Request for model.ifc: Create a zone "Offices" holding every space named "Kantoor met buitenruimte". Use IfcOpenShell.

First a look at what the model holds.

```python
import ifcopenshell

model = ifcopenshell.open("model.ifc")
print(model.schema)
seen = {}
for space in model.by_type("IfcSpace"):
    seen[space.LongName] = seen.get(space.LongName, 0) + 1
for name, count in sorted(seen.items(), key=str):
    print(count, "x", name)
print("zones:", [z.Name for z in model.by_type("IfcZone")][:20])
```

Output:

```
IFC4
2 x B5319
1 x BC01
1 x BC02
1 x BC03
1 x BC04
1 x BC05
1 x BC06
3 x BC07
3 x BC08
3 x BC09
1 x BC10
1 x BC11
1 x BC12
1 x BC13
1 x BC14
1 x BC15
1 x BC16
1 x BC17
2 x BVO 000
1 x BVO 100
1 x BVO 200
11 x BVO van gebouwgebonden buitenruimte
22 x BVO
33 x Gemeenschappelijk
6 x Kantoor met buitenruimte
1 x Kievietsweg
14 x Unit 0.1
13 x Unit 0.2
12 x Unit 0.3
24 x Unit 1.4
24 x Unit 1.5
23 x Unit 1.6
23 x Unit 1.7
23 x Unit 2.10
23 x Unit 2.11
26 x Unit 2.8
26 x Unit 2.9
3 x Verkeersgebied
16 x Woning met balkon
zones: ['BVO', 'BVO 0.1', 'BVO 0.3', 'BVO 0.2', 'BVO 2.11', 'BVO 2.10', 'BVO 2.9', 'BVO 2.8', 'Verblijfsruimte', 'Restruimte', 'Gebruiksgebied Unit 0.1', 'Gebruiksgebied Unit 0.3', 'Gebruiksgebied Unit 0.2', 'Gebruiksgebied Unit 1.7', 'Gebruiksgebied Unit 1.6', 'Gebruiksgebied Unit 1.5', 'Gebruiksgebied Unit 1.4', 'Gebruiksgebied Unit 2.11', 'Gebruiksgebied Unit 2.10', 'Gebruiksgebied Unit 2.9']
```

```python
import ifcopenshell
import ifcopenshell.api.group
import ifcopenshell.api.root

model = ifcopenshell.open("model.ifc")

names = {"Kantoor met buitenruimte"}
spaces = [s for s in model.by_type("IfcSpace") if s.LongName in names]

zone = ifcopenshell.api.root.create_entity(model, ifc_class="IfcZone", name="Offices")
ifcopenshell.api.group.assign_group(model, products=spaces, group=zone)
print(len(spaces), "spaces in", zone.Name)

model.write("model_updated.ifc")
```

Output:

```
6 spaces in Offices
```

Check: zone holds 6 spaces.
